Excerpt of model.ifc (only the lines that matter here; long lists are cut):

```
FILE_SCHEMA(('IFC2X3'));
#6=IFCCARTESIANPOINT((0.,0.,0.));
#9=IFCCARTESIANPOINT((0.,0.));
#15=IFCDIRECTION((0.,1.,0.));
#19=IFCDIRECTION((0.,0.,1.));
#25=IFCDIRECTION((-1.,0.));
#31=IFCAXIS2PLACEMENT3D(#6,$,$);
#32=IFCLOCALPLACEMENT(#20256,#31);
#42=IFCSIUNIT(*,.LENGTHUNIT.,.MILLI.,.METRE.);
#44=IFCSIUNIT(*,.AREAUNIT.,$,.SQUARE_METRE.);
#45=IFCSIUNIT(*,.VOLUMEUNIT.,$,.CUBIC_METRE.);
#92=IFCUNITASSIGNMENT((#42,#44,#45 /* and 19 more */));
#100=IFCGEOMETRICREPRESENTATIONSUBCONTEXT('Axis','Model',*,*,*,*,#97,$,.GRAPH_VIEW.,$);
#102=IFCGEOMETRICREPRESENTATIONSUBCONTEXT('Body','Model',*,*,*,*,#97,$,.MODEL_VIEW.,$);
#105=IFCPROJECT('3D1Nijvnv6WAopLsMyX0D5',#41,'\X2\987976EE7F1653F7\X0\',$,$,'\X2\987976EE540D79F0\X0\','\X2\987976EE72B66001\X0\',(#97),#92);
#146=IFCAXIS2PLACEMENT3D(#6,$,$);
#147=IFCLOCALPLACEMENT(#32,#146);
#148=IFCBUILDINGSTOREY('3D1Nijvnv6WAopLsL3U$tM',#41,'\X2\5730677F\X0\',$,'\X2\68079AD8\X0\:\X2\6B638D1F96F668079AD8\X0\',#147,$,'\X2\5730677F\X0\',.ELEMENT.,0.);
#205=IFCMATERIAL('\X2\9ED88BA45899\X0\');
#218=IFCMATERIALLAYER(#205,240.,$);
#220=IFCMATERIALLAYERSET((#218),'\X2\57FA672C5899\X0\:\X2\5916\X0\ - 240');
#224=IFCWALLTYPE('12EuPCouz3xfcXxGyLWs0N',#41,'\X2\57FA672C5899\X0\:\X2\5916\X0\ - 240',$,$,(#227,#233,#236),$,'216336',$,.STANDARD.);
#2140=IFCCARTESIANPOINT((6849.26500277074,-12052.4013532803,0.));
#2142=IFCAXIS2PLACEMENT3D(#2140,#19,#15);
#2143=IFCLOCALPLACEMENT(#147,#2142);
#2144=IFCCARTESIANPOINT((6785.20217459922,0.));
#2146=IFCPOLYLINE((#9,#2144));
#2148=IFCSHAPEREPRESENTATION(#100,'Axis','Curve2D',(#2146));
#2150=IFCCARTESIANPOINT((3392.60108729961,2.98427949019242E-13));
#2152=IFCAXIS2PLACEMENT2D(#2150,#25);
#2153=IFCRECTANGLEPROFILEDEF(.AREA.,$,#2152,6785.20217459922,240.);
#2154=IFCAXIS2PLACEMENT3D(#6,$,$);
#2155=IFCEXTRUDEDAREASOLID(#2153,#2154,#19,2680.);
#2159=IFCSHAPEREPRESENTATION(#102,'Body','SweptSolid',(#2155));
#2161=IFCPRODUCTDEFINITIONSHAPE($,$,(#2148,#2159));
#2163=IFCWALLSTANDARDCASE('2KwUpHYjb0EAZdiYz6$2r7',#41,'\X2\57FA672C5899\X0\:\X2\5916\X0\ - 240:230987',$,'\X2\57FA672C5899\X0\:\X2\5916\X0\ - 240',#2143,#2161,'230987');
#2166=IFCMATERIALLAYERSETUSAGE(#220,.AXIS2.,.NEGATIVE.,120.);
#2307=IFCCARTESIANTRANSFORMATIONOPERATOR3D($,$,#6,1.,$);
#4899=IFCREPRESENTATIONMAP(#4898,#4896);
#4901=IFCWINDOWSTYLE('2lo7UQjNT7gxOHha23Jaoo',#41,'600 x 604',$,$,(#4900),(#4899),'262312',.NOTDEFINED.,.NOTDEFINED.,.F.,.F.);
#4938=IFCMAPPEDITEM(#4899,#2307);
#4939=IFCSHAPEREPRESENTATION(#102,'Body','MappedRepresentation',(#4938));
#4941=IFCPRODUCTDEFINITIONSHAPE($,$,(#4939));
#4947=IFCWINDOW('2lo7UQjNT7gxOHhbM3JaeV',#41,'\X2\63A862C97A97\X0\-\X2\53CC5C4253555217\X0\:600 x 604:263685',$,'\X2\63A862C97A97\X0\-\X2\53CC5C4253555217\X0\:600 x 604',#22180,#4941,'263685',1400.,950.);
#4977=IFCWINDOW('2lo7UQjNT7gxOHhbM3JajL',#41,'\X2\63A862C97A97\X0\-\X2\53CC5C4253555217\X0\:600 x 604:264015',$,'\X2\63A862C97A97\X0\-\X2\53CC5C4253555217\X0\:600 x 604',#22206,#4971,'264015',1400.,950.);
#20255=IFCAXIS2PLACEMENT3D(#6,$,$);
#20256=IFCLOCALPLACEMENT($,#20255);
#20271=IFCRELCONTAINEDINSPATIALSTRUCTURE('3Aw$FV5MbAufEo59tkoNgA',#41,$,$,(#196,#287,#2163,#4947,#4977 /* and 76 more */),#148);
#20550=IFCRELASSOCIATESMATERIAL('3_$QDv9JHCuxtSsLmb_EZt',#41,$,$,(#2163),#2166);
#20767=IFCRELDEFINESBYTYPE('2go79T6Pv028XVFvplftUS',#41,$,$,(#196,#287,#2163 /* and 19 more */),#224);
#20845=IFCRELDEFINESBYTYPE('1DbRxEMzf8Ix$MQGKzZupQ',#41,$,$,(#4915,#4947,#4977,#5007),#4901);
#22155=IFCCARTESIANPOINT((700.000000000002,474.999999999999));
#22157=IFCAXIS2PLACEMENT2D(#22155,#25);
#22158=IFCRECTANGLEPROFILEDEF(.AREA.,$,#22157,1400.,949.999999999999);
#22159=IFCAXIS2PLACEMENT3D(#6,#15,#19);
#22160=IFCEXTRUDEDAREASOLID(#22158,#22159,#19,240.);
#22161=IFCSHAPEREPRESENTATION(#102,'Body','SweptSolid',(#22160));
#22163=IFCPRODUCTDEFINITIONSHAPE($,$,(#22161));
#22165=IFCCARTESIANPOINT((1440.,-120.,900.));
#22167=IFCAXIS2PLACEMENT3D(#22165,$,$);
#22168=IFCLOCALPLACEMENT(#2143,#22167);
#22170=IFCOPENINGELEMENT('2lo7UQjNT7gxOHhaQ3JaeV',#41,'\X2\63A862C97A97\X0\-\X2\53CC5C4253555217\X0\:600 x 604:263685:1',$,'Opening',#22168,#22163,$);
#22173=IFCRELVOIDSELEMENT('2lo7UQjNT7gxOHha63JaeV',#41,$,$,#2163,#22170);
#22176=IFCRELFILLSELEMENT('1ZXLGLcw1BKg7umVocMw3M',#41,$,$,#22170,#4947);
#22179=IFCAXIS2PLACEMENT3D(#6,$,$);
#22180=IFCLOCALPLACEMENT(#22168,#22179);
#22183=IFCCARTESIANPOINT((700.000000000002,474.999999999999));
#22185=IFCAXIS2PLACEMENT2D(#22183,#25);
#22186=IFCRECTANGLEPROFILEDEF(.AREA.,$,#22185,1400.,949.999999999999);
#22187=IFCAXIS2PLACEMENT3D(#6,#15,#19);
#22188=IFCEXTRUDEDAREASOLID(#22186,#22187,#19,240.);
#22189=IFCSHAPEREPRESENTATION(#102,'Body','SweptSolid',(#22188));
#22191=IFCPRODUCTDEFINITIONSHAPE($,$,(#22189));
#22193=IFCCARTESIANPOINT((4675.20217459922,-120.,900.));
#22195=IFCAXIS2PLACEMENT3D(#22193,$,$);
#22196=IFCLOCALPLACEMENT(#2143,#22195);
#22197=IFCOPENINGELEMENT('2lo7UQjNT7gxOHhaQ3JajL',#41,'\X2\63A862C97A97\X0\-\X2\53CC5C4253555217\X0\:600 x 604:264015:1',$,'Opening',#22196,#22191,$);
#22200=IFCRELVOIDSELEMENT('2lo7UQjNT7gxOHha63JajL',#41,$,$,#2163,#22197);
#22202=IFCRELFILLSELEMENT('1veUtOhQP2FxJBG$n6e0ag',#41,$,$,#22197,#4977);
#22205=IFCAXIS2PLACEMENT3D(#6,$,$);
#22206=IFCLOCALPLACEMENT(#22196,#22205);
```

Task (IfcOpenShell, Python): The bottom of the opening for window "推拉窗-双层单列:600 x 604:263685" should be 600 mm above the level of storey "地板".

```python
import numpy as np
import ifcopenshell
import ifcopenshell.api.geometry
import ifcopenshell.geom
import ifcopenshell.util.element
import ifcopenshell.util.placement
import ifcopenshell.util.shape
import ifcopenshell.util.unit

model = ifcopenshell.open("model.ifc")
unit_scale = ifcopenshell.util.unit.calculate_unit_scale(model)

window = model.by_guid("2lo7UQjNT7gxOHhbM3JaeV")
opening = window.FillsVoids[0].RelatingOpeningElement
storey = ifcopenshell.util.element.get_container(window, ifc_class="IfcBuildingStorey")
level = ifcopenshell.util.placement.get_local_placement(storey.ObjectPlacement)[2, 3]

# The opening's origin need not be at the sill, so measure its lowest point.
shape = ifcopenshell.geom.create_shape(ifcopenshell.geom.settings(), opening)
bottom = ifcopenshell.util.shape.get_shape_bottom_elevation(shape, shape.geometry) / unit_scale
dz = level + 600.0 - bottom

shift = np.array([0.0, 0.0, dz])
# The window is placed relative to its opening, so it follows when the opening moves.
matrix = ifcopenshell.util.placement.get_local_placement(opening.ObjectPlacement)
matrix[:3, 3] += shift
ifcopenshell.api.geometry.edit_object_placement(
    model, product=opening, matrix=matrix, is_si=False, should_transform_children=True
)

print(f"moved by {dz * unit_scale:+.3f} m")

model.write("model_updated.ifc")
```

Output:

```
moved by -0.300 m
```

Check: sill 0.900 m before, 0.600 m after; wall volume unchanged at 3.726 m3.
